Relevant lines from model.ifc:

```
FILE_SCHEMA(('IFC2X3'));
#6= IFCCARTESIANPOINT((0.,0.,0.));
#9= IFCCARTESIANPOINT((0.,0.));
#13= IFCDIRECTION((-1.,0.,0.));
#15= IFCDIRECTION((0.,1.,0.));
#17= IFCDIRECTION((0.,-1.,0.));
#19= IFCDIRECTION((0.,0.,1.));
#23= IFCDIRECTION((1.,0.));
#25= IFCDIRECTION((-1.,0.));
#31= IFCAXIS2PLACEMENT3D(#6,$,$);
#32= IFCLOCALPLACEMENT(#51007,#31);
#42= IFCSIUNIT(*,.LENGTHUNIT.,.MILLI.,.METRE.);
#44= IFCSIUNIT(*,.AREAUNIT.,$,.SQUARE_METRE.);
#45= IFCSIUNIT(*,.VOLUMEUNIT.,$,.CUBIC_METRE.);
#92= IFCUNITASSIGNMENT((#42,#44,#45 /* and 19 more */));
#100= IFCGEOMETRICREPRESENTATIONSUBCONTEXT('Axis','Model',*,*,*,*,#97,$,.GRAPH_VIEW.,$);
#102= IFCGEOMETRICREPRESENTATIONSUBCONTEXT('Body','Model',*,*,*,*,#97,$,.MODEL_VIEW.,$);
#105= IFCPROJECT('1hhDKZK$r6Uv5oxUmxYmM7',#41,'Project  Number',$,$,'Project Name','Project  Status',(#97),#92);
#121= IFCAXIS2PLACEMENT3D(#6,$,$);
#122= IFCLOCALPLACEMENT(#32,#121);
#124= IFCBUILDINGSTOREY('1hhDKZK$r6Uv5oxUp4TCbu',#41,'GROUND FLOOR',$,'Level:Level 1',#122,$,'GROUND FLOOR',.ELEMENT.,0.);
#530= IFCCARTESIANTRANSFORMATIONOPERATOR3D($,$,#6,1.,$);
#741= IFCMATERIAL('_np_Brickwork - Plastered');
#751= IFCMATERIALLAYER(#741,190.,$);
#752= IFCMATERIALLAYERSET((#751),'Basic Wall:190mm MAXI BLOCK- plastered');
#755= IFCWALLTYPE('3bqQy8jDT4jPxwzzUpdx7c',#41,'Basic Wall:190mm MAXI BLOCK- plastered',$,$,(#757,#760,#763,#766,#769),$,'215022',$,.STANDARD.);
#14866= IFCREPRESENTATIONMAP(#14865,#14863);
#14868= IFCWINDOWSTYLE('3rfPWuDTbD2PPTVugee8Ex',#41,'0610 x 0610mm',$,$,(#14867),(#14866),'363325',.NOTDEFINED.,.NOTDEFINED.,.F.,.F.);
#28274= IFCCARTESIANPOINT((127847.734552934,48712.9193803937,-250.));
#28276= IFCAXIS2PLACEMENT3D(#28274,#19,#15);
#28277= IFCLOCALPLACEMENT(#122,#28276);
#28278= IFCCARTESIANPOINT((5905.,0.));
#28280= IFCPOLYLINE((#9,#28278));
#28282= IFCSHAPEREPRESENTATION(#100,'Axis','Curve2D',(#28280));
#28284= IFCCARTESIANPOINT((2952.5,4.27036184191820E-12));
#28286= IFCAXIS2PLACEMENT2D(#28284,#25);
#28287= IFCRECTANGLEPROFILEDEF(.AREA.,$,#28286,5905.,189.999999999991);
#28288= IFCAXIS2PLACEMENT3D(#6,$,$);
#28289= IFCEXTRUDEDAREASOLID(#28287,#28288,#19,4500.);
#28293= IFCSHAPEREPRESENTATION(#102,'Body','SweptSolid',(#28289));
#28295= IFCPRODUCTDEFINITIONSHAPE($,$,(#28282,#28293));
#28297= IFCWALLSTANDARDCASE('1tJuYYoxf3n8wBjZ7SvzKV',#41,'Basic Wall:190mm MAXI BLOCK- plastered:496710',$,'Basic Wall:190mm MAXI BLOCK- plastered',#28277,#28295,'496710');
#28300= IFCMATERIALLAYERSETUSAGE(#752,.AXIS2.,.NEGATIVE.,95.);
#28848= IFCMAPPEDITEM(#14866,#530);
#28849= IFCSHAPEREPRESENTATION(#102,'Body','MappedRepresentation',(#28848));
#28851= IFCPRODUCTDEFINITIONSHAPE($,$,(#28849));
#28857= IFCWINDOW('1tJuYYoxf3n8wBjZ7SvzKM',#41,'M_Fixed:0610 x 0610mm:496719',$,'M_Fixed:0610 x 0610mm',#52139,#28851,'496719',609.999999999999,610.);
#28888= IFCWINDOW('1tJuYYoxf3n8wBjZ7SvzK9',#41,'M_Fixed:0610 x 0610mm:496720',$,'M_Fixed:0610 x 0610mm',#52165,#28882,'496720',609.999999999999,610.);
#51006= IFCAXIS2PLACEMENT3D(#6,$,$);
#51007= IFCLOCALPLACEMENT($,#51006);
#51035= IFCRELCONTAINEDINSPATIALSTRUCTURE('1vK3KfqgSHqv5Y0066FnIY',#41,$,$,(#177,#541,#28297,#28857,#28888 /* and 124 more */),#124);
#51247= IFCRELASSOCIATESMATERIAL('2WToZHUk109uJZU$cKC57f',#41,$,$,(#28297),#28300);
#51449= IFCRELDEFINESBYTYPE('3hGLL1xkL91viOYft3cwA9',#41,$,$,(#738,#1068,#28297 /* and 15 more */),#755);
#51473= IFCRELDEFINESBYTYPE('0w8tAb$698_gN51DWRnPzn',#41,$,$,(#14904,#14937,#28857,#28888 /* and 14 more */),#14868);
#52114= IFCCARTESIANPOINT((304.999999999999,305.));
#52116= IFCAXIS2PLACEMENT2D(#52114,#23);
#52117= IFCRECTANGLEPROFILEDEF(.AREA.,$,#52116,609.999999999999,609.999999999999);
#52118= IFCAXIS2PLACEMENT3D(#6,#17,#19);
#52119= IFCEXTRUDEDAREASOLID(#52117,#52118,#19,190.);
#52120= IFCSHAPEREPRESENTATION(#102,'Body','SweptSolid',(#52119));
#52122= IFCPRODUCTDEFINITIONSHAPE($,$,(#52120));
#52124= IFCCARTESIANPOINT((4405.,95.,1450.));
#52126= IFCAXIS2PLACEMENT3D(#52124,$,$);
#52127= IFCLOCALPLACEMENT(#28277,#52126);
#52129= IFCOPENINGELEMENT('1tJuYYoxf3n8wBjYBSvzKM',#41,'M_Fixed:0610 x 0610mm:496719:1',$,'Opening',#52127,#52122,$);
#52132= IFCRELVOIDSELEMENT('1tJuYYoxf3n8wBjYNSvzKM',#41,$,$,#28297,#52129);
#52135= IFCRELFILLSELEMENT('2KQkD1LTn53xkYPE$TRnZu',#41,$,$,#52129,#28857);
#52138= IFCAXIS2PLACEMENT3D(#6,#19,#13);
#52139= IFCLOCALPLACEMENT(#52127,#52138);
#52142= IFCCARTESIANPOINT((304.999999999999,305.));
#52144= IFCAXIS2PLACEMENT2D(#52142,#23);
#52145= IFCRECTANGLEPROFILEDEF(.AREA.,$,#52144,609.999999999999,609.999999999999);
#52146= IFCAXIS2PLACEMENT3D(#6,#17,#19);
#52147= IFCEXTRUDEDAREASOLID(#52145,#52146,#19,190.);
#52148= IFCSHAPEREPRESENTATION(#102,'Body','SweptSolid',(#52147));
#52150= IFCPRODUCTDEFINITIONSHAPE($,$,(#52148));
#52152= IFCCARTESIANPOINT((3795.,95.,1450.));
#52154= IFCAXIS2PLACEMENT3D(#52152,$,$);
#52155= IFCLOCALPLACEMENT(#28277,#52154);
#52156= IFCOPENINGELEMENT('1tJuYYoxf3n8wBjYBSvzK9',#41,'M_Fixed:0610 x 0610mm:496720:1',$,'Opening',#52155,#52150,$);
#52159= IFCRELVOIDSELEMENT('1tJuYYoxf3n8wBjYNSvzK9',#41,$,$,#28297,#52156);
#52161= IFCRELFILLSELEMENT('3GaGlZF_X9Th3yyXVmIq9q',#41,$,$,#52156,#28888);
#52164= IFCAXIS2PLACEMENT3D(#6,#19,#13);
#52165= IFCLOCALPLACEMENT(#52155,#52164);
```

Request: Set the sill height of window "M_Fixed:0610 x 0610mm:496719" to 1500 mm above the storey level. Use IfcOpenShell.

```python
import numpy as np
import ifcopenshell
import ifcopenshell.api.geometry
import ifcopenshell.geom
import ifcopenshell.util.element
import ifcopenshell.util.placement
import ifcopenshell.util.shape
import ifcopenshell.util.unit

model = ifcopenshell.open("model.ifc")
unit_scale = ifcopenshell.util.unit.calculate_unit_scale(model)

window = model.by_guid("1tJuYYoxf3n8wBjZ7SvzKM")
opening = window.FillsVoids[0].RelatingOpeningElement
storey = ifcopenshell.util.element.get_container(window, ifc_class="IfcBuildingStorey")
level = ifcopenshell.util.placement.get_local_placement(storey.ObjectPlacement)[2, 3]

# The opening's origin need not be at the sill, so measure its lowest point.
shape = ifcopenshell.geom.create_shape(ifcopenshell.geom.settings(), opening)
bottom = ifcopenshell.util.shape.get_shape_bottom_elevation(shape, shape.geometry) / unit_scale
dz = level + 1.5 / unit_scale - bottom

shift = np.array([0.0, 0.0, dz])
# The window is placed relative to its opening, so it follows when the opening moves.
matrix = ifcopenshell.util.placement.get_local_placement(opening.ObjectPlacement)
matrix[:3, 3] += shift
ifcopenshell.api.geometry.edit_object_placement(
    model, product=opening, matrix=matrix, is_si=False, should_transform_children=True
)

print(f"moved by {dz * unit_scale:+.3f} m")

model.write("model-out.ifc")
```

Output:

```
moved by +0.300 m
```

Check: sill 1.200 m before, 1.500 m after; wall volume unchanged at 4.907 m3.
